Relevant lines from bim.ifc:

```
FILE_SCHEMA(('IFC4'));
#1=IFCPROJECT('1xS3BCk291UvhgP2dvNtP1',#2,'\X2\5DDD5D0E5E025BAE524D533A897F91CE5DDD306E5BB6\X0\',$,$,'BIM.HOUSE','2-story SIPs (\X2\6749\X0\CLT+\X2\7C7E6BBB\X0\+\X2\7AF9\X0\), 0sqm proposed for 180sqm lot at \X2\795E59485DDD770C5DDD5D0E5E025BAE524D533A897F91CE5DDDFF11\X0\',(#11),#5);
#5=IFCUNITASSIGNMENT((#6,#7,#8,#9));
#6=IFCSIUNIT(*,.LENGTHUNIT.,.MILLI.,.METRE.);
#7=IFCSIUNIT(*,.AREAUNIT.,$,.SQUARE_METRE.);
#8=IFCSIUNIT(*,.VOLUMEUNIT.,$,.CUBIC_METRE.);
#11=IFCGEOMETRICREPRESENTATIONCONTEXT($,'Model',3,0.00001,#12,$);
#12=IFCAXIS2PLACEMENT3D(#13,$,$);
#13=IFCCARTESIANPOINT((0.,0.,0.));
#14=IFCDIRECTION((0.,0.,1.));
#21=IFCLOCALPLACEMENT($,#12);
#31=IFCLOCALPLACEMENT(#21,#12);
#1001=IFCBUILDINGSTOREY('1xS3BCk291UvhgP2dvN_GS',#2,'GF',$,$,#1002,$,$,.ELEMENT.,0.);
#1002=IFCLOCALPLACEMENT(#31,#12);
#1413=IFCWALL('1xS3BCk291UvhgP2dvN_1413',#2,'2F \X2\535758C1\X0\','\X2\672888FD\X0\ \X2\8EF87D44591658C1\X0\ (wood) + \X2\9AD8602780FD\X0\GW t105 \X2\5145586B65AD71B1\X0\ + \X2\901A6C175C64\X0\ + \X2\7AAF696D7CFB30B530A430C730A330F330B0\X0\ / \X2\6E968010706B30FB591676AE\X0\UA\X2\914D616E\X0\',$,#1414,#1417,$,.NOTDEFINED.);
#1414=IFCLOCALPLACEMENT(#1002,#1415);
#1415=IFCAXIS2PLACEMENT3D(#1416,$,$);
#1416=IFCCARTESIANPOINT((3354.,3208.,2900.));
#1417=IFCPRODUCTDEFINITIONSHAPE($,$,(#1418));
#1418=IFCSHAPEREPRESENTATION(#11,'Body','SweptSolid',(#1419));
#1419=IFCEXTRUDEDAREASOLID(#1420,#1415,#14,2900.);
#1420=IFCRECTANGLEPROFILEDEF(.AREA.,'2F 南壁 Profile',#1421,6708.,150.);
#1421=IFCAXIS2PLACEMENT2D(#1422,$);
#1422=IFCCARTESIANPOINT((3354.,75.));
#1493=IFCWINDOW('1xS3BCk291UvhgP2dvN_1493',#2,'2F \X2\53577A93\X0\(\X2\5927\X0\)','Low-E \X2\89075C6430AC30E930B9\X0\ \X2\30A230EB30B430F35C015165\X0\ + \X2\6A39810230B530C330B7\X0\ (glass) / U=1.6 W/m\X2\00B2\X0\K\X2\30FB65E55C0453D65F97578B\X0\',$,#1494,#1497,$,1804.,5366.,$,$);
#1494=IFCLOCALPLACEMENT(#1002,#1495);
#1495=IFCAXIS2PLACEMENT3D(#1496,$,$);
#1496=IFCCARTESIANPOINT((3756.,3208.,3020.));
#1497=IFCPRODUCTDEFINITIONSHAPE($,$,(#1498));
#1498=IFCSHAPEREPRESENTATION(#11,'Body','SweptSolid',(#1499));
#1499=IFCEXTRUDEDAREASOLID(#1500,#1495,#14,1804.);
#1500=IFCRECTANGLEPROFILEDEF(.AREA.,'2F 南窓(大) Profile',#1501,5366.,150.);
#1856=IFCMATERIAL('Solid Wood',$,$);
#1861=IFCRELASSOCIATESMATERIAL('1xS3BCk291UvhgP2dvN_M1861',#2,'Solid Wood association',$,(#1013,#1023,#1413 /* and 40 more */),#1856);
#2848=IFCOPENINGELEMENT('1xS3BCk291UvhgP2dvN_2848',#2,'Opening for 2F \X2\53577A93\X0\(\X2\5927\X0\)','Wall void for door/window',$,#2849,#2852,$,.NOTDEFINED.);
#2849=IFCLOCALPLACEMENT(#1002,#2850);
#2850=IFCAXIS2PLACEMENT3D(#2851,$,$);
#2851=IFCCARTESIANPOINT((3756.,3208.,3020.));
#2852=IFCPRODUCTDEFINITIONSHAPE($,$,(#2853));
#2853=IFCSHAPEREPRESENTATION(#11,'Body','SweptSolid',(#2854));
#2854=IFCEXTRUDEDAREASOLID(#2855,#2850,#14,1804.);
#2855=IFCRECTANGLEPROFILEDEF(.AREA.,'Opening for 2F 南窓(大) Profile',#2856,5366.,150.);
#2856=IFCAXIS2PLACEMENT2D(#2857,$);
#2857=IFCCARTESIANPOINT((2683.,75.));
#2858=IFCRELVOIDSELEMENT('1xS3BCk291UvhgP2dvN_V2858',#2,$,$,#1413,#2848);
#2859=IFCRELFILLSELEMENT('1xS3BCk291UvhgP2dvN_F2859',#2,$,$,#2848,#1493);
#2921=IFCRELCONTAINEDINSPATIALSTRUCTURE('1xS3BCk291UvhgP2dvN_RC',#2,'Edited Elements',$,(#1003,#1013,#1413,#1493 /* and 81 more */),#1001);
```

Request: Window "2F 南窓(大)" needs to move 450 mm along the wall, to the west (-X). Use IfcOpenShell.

```python
import ifcopenshell
import ifcopenshell.api.geometry
import ifcopenshell.util.placement

model = ifcopenshell.open("bim.ifc")

window = model.by_guid("1xS3BCk291UvhgP2dvN_1493")
opening = window.FillsVoids[0].RelatingOpeningElement
wall = opening.VoidsElements[0].RelatingBuildingElement

wall_matrix = ifcopenshell.util.placement.get_local_placement(wall.ObjectPlacement)
shift = wall_matrix[:3, 0] * -450.0
before = ifcopenshell.util.placement.get_local_placement(window.ObjectPlacement)[:3, 3].copy()

# The window is not placed relative to its opening, so move both.
for product in (opening, window):
    matrix = ifcopenshell.util.placement.get_local_placement(product.ObjectPlacement)
    matrix[:3, 3] += shift
    ifcopenshell.api.geometry.edit_object_placement(model, product=product, matrix=matrix, is_si=False)

after = ifcopenshell.util.placement.get_local_placement(window.ObjectPlacement)[:3, 3]
print("window moved by", (after - before).round(3) + 0.0)

model.write("bim_updated.ifc")
```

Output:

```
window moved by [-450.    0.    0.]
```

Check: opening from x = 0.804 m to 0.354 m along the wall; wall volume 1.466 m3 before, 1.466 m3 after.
